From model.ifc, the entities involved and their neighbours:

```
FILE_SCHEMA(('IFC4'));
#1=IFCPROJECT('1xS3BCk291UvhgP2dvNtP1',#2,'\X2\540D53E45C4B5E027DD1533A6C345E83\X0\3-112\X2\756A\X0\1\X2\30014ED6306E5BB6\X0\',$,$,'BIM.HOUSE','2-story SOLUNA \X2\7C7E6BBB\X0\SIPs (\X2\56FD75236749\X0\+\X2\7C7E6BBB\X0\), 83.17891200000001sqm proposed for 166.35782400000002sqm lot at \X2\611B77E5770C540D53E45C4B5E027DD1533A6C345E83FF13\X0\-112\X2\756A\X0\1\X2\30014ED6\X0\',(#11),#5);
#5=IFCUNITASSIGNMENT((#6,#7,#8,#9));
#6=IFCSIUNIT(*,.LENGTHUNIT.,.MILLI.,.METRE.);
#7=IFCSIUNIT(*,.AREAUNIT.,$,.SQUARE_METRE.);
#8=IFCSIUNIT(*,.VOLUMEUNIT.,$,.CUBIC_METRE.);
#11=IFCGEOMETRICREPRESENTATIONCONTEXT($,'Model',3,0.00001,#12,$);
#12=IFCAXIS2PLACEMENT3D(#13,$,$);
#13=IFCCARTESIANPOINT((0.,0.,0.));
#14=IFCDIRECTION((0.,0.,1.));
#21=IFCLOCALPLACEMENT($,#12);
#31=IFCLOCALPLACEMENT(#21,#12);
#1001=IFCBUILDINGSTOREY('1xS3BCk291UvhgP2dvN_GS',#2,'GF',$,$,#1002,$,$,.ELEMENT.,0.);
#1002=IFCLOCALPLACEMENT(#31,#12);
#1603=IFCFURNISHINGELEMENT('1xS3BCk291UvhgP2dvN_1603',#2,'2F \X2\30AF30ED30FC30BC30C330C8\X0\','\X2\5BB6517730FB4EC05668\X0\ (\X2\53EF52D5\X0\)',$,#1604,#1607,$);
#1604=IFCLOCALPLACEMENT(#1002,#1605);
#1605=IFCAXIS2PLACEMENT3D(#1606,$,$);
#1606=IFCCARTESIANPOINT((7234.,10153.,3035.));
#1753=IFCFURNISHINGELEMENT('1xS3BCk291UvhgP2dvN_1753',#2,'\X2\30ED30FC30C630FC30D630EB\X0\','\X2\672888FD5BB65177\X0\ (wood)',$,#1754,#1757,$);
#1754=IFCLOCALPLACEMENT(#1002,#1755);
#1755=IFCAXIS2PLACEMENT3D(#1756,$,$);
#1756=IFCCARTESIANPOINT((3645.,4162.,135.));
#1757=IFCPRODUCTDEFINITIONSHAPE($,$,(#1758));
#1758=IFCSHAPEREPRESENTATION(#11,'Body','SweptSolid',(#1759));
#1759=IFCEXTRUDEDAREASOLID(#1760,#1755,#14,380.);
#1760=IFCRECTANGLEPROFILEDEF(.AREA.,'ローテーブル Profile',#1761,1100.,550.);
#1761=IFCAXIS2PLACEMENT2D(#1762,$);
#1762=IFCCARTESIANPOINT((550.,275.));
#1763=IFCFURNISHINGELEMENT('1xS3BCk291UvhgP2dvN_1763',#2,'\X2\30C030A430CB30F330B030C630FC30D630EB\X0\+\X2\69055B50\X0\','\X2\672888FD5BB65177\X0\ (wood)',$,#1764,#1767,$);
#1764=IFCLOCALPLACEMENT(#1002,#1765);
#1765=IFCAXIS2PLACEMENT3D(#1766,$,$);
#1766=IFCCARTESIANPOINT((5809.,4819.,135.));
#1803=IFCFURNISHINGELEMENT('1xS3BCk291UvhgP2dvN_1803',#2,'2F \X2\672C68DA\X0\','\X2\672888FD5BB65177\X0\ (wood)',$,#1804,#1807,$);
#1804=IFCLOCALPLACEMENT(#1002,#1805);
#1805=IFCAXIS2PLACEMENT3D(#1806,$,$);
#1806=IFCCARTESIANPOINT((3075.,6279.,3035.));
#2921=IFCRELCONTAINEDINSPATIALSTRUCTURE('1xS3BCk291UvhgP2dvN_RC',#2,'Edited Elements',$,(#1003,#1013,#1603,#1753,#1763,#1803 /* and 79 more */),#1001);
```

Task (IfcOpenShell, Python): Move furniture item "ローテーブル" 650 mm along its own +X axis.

```python
import ifcopenshell
import ifcopenshell.api.geometry
import ifcopenshell.util.placement
import ifcopenshell.util.unit

model = ifcopenshell.open("model.ifc")
unit_scale = ifcopenshell.util.unit.calculate_unit_scale(model)

item = model.by_guid("1xS3BCk291UvhgP2dvN_1753")
matrix = ifcopenshell.util.placement.get_local_placement(item.ObjectPlacement)
matrix[:3, 3] += matrix[:3, 0] * 0.65 / unit_scale
ifcopenshell.api.geometry.edit_object_placement(model, product=item, matrix=matrix, is_si=False)

print(ifcopenshell.util.placement.get_local_placement(item.ObjectPlacement).round(3) + 0.0)

model.write("model-out.ifc")
```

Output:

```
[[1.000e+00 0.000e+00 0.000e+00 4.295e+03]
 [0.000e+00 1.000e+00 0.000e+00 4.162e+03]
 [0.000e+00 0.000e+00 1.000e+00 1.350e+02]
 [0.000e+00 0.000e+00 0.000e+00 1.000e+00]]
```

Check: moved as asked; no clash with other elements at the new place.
